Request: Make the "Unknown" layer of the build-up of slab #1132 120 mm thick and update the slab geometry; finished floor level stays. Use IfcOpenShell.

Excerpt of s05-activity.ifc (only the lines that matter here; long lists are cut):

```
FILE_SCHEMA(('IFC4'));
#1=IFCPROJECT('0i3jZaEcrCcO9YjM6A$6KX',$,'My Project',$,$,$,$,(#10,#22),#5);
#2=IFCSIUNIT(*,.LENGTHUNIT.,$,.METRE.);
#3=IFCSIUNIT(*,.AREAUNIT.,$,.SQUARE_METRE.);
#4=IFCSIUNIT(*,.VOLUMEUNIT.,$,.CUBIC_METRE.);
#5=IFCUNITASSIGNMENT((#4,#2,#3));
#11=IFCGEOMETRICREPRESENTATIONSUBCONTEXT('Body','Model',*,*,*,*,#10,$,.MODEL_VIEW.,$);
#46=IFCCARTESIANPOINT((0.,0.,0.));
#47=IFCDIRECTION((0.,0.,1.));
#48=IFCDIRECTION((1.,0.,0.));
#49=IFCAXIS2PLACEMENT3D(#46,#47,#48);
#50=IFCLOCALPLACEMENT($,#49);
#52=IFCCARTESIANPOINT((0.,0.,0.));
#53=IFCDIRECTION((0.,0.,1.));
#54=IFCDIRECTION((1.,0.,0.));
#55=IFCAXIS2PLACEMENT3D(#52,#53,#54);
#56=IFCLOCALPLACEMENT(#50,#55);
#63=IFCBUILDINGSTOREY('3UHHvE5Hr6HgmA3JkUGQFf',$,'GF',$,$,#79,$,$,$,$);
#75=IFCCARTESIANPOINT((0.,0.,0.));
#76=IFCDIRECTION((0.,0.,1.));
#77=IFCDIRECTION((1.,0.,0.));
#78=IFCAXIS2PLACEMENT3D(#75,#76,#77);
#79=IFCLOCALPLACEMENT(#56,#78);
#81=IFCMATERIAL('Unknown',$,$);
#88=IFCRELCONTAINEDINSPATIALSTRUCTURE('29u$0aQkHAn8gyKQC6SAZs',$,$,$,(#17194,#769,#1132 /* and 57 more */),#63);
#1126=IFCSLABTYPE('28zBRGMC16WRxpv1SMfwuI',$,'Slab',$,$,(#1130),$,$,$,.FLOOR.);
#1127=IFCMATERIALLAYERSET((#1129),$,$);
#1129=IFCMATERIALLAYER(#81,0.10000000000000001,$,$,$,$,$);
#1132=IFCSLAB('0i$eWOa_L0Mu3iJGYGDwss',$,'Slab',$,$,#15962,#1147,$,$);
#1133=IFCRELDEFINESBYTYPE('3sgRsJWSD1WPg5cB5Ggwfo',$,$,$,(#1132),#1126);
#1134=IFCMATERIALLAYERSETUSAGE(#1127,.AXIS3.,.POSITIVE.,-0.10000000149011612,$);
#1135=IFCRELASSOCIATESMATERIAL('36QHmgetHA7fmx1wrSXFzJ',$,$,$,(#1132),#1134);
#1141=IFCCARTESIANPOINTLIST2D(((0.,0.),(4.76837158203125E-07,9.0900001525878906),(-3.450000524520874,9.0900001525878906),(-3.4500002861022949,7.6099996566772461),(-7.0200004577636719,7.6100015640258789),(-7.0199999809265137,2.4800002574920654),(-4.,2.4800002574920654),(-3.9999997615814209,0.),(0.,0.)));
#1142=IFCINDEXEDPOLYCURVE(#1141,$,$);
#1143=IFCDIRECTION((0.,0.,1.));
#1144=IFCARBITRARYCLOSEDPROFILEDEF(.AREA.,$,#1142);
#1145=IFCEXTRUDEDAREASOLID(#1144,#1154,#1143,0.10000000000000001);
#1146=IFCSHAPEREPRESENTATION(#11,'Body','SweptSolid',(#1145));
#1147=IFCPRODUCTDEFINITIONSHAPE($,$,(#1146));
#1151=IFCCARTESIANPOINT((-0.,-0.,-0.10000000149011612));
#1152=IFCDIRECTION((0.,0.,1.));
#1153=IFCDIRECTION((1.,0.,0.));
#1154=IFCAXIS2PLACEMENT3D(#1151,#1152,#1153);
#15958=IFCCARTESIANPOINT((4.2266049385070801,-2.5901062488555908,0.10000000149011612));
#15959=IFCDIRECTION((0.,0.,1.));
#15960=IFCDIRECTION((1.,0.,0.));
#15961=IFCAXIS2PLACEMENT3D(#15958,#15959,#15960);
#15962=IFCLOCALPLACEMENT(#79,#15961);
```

```python
import ifcopenshell
import ifcopenshell.util.element
import ifcopenshell.util.representation
import ifcopenshell.util.unit

model = ifcopenshell.open("s05-activity.ifc")
unit_scale = ifcopenshell.util.unit.calculate_unit_scale(model)

layer_set = model.by_id(1127)
layer = next(l for l in layer_set.MaterialLayers if l.Material and l.Material.Name == "Unknown")
change = 0.12 / unit_scale - layer.LayerThickness
layer.LayerThickness += change

# Geometry does not follow the layer set by itself.
slabs = [e for e in ifcopenshell.util.element.get_elements_by_material(model, layer_set) if e.is_a("IfcSlab")]
for slab in sorted(slabs, key=lambda e: e.id()):
    body = ifcopenshell.util.representation.get_representation(slab, "Model", "Body")
    solid = body.Items[0]
    old_depth = solid.Depth
    solid.Depth += change
    # Extruded upwards: lower the start of the extrusion so the top stays.
    x, y, z = solid.Position.Location.Coordinates
    solid.Position.Location = model.createIfcCartesianPoint((x, y, z - change))
    print(slab.id(), f"{old_depth:g} -> {solid.Depth:g}")

# The layers are counted up from the underside, which has moved.
for usage in {ifcopenshell.util.element.get_material(slab) for slab in slabs}:
    usage.OffsetFromReferenceLine -= change

model.write("s05-activity_edited.ifc")
```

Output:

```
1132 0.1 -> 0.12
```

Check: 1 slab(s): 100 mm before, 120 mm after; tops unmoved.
